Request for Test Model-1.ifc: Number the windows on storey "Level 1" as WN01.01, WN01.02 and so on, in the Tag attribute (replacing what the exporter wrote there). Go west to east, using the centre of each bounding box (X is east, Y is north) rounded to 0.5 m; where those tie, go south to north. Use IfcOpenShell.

First a look at what the model holds.

```python
import ifcopenshell
import ifcopenshell.util.element
import ifcopenshell.util.placement

model = ifcopenshell.open("Test Model-1.ifc")
print(model.schema)
storey = next(s for s in model.by_type("IfcBuildingStorey") if s.Name == "Level 1")
windows = [e for e in ifcopenshell.util.element.get_decomposition(storey) if e.is_a("IfcWindow")]
for e in sorted(windows, key=lambda e: e.id()):
    origin = ifcopenshell.util.placement.get_local_placement(e.ObjectPlacement)[:3, 3]
    print(e.id(), e.Tag, e.Name, origin.round(2) + 0.0, sep=" | ")
```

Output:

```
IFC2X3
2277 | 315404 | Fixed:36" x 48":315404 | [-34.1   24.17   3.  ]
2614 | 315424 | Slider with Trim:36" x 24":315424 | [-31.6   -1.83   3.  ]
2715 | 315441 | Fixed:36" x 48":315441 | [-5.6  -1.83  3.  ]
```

```python
import ifcopenshell
import ifcopenshell.geom
import ifcopenshell.util.element
import ifcopenshell.util.shape

model = ifcopenshell.open("Test Model-1.ifc")
settings = ifcopenshell.geom.settings()
settings.set("use-world-coords", True)


def centre(element):
    shape = ifcopenshell.geom.create_shape(settings, element)
    return ifcopenshell.util.shape.get_bbox_centroid(shape.geometry)


storey = next(s for s in model.by_type("IfcBuildingStorey") if s.Name == "Level 1")
windows = [e for e in ifcopenshell.util.element.get_decomposition(storey) if e.is_a("IfcWindow")]

# Insertion points can sit at a corner or the storey origin, so sort by the geometry (in metres).
centres = {e: centre(e) for e in windows}
windows.sort(key=lambda e: (round(centres[e][0] / 0.5), centres[e][1]))

for i, e in enumerate(windows, start=1):
    number = f"WN01.{i:02d}"
    e.Tag = number
    print(e.id(), number)

model.write("Test Model-1-out.ifc")
```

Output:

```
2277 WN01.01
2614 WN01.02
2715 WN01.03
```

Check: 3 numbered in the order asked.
